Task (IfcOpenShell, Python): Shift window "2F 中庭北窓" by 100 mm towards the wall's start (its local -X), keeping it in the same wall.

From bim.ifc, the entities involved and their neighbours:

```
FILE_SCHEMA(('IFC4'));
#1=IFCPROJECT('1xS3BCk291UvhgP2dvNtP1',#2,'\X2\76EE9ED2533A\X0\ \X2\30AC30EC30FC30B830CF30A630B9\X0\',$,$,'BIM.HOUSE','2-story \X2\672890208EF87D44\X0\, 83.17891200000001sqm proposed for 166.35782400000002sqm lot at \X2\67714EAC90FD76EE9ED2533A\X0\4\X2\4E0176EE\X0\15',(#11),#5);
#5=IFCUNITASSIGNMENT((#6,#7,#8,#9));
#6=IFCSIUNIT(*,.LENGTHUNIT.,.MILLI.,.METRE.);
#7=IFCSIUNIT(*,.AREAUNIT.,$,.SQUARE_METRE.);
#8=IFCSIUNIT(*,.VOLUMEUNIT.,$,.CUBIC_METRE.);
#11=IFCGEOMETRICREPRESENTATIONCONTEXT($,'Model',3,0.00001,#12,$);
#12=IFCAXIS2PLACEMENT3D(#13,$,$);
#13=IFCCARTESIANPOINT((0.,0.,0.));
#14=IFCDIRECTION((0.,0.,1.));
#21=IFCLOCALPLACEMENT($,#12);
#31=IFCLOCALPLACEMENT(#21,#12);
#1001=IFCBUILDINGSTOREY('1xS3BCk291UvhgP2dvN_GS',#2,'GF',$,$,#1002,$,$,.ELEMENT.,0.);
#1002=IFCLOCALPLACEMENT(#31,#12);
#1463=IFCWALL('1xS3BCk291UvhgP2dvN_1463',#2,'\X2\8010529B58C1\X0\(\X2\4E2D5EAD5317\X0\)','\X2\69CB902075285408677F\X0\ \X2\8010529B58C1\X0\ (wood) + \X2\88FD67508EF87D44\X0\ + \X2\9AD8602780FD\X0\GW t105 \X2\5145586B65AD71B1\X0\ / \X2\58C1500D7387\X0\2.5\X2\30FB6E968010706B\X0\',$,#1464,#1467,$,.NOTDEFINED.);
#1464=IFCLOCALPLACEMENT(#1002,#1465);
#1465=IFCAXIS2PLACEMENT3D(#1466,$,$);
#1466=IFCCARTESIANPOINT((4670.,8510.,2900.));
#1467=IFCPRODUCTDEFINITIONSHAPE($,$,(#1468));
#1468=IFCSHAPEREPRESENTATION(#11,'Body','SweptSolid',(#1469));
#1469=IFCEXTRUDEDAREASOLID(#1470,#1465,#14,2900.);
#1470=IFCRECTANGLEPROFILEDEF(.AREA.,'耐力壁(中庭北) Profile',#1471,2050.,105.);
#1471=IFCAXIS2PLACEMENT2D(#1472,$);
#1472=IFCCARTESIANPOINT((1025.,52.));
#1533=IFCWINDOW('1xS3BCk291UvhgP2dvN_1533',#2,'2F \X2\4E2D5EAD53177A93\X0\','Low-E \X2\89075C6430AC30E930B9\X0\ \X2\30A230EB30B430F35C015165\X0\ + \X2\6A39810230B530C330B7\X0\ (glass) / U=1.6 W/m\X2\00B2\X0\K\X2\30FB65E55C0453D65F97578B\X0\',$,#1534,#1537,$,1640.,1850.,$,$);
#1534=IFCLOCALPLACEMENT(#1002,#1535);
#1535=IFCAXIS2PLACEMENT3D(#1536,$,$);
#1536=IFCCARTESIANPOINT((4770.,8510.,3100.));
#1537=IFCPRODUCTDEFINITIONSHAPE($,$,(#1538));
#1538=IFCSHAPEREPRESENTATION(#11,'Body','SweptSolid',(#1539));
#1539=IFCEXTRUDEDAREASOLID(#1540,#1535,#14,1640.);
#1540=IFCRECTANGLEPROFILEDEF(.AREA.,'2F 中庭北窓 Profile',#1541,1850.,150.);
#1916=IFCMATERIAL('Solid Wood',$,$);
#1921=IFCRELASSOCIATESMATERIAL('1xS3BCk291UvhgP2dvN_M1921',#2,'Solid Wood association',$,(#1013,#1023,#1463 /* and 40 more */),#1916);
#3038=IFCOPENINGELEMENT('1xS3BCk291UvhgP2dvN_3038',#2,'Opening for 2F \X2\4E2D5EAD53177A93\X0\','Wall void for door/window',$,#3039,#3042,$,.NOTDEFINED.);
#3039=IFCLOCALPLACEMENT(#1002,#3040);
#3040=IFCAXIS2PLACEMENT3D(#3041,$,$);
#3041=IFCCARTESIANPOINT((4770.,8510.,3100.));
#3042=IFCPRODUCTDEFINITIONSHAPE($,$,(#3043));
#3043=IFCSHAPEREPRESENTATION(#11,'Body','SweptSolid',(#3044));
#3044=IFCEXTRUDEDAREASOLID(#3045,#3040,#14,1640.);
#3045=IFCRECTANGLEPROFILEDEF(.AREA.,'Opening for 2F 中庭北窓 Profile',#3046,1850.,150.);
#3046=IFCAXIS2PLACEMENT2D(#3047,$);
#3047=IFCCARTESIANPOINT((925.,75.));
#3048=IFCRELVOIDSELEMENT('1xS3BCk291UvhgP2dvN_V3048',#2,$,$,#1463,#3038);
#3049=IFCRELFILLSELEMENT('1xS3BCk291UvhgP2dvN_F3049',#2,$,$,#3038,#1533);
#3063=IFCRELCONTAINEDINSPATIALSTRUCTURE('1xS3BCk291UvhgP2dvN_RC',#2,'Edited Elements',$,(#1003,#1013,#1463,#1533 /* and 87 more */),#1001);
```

```python
import ifcopenshell
import ifcopenshell.api.geometry
import ifcopenshell.util.placement
import ifcopenshell.util.unit

model = ifcopenshell.open("bim.ifc")
unit_scale = ifcopenshell.util.unit.calculate_unit_scale(model)

window = model.by_guid("1xS3BCk291UvhgP2dvN_1533")
opening = window.FillsVoids[0].RelatingOpeningElement
wall = opening.VoidsElements[0].RelatingBuildingElement

wall_matrix = ifcopenshell.util.placement.get_local_placement(wall.ObjectPlacement)
shift = wall_matrix[:3, 0] * -0.1 / unit_scale
before = ifcopenshell.util.placement.get_local_placement(window.ObjectPlacement)[:3, 3].copy()

# The window is not placed relative to its opening, so move both.
for product in (opening, window):
    matrix = ifcopenshell.util.placement.get_local_placement(product.ObjectPlacement)
    matrix[:3, 3] += shift
    ifcopenshell.api.geometry.edit_object_placement(model, product=product, matrix=matrix, is_si=False)

after = ifcopenshell.util.placement.get_local_placement(window.ObjectPlacement)[:3, 3]
print("window moved by", (after - before).round(3) + 0.0)

model.write("bim_v2.ifc")
```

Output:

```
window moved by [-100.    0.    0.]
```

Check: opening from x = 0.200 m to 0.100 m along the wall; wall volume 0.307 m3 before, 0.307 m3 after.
